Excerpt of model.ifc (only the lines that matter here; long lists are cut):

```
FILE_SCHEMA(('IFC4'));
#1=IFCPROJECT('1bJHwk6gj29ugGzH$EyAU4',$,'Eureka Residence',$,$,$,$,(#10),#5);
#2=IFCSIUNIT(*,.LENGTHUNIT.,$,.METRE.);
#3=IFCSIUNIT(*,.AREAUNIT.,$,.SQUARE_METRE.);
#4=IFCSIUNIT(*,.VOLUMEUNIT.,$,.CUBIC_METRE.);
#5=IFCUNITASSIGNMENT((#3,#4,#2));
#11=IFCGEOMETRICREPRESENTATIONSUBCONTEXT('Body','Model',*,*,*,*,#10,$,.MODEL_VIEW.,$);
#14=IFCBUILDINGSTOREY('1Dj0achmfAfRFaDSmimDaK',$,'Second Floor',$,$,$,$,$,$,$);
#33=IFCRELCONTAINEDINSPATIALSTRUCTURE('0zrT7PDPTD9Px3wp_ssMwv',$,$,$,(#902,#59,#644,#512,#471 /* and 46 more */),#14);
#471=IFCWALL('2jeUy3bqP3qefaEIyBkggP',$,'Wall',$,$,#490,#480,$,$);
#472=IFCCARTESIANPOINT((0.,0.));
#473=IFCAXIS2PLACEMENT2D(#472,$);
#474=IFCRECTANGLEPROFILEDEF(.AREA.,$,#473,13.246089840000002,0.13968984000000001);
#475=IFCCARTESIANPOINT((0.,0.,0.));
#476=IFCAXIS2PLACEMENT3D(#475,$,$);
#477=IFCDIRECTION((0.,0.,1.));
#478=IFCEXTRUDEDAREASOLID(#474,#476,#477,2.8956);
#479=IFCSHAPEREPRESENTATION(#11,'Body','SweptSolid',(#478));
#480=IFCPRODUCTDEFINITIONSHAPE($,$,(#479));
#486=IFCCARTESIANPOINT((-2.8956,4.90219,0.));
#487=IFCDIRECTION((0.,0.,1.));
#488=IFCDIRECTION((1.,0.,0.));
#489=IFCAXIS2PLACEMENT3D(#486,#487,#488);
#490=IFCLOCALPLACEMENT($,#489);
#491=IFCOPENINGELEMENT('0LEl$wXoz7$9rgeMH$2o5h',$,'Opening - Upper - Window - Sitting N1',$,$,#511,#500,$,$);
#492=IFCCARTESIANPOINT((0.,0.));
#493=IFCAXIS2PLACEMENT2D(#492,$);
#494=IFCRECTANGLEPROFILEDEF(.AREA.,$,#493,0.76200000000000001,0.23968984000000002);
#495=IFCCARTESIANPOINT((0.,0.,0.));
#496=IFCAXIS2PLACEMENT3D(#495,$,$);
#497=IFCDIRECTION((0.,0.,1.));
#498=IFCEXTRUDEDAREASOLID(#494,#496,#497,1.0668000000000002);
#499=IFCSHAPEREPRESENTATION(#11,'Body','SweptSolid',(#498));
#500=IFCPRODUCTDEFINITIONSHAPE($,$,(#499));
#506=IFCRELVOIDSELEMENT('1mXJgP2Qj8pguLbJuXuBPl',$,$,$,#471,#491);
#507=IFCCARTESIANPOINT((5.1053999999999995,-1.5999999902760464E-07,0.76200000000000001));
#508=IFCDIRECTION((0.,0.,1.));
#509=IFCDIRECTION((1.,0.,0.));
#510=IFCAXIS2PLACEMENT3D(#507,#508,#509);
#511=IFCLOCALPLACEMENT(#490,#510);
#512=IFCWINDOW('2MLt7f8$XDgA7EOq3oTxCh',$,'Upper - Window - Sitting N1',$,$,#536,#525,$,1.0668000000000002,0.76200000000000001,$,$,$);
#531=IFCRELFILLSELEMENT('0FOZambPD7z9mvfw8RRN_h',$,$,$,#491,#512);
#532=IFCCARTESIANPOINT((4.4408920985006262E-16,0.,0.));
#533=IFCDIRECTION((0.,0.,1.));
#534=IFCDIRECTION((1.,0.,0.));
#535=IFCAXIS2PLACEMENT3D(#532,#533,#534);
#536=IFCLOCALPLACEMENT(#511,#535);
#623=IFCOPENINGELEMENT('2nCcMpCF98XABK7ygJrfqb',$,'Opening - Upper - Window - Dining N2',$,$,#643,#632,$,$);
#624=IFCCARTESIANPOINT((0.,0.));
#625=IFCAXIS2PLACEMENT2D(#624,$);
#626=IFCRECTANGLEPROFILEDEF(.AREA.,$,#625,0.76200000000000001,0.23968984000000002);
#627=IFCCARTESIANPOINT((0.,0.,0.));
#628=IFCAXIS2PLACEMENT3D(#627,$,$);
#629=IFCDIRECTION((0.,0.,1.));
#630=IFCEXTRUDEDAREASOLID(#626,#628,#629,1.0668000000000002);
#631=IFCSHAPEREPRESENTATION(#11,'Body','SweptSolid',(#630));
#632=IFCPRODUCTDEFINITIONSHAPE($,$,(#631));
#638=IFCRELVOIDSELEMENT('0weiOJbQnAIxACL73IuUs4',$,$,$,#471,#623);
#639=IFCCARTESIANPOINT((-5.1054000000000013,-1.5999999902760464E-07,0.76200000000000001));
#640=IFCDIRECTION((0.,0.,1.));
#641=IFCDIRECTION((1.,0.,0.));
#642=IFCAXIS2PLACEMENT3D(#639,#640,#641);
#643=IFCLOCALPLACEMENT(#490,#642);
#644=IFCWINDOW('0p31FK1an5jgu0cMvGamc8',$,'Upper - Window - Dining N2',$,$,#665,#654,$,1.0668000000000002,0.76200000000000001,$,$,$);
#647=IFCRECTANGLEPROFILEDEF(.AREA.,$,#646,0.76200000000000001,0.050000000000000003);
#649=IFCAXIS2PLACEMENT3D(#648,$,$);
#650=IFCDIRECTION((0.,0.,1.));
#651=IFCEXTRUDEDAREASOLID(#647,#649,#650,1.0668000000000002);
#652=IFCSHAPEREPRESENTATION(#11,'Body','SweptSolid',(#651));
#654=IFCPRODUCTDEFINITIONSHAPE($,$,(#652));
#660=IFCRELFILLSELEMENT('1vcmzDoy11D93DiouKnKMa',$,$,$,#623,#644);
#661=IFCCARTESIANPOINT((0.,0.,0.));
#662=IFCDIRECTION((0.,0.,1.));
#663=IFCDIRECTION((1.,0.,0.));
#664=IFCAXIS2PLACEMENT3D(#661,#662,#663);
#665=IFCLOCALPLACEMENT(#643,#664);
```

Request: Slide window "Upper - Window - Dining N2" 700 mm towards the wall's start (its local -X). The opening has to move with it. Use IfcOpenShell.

```python
import ifcopenshell
import ifcopenshell.api.geometry
import ifcopenshell.util.placement

model = ifcopenshell.open("model.ifc")

window = model.by_guid("0p31FK1an5jgu0cMvGamc8")
opening = window.FillsVoids[0].RelatingOpeningElement
wall = opening.VoidsElements[0].RelatingBuildingElement

wall_matrix = ifcopenshell.util.placement.get_local_placement(wall.ObjectPlacement)
shift = wall_matrix[:3, 0] * -0.7
before = ifcopenshell.util.placement.get_local_placement(window.ObjectPlacement)[:3, 3].copy()

# The window is placed relative to its opening, so it follows when the opening moves.
matrix = ifcopenshell.util.placement.get_local_placement(opening.ObjectPlacement)
matrix[:3, 3] += shift
ifcopenshell.api.geometry.edit_object_placement(
    model, product=opening, matrix=matrix, is_si=False, should_transform_children=True
)

after = ifcopenshell.util.placement.get_local_placement(window.ObjectPlacement)[:3, 3]
print("window moved by", (after - before).round(3) + 0.0)

model.write("model_rev.ifc")
```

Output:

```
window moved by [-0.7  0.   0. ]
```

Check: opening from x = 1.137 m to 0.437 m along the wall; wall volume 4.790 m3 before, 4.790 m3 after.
